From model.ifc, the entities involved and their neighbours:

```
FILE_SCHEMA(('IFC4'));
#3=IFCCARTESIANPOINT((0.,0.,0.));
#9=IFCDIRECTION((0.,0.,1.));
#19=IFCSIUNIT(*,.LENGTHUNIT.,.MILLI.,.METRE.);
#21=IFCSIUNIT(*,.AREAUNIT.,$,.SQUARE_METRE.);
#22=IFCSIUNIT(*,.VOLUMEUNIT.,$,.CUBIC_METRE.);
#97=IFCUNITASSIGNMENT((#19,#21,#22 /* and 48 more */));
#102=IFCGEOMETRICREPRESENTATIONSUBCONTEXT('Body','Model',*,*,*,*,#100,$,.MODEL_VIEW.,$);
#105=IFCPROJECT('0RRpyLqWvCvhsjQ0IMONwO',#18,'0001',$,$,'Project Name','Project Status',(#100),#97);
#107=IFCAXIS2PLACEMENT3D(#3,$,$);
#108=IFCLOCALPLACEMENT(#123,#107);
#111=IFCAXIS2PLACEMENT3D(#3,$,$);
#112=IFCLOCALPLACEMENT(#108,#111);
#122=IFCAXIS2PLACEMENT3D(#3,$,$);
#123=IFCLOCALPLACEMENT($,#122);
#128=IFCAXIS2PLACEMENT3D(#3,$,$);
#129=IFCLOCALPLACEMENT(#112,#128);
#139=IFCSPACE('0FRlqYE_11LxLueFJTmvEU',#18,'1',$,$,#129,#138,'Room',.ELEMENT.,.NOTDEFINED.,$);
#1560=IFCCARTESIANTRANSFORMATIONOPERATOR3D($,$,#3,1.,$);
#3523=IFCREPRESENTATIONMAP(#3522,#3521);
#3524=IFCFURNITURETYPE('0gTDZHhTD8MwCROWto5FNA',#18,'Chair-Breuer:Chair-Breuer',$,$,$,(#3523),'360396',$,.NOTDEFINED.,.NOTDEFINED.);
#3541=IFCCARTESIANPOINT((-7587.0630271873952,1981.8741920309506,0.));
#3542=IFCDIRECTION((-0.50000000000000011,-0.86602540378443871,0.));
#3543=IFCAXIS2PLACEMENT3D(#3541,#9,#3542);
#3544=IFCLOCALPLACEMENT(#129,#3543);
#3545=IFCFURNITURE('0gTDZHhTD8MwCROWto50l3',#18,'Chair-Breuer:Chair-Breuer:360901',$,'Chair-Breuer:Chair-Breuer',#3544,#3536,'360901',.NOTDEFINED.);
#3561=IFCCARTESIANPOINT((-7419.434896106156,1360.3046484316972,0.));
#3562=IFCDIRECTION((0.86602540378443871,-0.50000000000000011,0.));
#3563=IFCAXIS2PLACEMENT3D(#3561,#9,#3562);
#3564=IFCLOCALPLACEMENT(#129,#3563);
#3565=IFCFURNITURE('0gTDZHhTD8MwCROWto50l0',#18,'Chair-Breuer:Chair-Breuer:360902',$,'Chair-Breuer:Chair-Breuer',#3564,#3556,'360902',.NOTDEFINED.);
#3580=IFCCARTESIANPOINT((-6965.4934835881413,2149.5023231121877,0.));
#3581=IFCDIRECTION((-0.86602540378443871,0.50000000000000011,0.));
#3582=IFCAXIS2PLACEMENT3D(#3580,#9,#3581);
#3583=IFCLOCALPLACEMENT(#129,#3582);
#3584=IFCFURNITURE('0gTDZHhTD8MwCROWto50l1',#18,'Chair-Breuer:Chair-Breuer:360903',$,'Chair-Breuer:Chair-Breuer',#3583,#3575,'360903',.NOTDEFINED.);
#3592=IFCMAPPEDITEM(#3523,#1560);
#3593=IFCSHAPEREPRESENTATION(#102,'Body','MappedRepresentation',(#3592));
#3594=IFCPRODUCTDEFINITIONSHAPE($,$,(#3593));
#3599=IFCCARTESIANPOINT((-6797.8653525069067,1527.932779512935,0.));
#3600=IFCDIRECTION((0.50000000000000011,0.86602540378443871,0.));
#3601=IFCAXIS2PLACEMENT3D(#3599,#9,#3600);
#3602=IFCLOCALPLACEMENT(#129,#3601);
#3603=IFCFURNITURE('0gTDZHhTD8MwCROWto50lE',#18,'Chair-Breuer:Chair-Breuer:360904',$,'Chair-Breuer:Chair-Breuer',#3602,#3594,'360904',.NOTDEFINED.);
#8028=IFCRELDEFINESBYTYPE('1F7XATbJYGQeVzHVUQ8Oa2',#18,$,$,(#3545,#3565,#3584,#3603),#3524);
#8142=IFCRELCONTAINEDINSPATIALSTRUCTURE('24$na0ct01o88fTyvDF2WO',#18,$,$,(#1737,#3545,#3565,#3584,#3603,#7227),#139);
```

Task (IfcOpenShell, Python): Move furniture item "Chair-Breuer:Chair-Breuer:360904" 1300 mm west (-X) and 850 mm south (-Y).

```python
import ifcopenshell
import ifcopenshell.api.geometry
import ifcopenshell.util.placement
import ifcopenshell.util.unit

model = ifcopenshell.open("model.ifc")
unit_scale = ifcopenshell.util.unit.calculate_unit_scale(model)

item = model.by_id(3603)
matrix = ifcopenshell.util.placement.get_local_placement(item.ObjectPlacement)
matrix[0, 3] -= 1.3 / unit_scale
matrix[1, 3] -= 0.85 / unit_scale
ifcopenshell.api.geometry.edit_object_placement(model, product=item, matrix=matrix, is_si=False)

print(ifcopenshell.util.placement.get_local_placement(item.ObjectPlacement).round(3) + 0.0)

model.write("model-out.ifc")
```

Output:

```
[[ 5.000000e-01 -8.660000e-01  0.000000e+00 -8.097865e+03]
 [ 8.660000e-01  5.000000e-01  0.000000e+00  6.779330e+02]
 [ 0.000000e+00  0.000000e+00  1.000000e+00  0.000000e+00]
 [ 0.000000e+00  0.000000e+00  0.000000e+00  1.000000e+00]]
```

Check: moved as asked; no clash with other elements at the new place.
